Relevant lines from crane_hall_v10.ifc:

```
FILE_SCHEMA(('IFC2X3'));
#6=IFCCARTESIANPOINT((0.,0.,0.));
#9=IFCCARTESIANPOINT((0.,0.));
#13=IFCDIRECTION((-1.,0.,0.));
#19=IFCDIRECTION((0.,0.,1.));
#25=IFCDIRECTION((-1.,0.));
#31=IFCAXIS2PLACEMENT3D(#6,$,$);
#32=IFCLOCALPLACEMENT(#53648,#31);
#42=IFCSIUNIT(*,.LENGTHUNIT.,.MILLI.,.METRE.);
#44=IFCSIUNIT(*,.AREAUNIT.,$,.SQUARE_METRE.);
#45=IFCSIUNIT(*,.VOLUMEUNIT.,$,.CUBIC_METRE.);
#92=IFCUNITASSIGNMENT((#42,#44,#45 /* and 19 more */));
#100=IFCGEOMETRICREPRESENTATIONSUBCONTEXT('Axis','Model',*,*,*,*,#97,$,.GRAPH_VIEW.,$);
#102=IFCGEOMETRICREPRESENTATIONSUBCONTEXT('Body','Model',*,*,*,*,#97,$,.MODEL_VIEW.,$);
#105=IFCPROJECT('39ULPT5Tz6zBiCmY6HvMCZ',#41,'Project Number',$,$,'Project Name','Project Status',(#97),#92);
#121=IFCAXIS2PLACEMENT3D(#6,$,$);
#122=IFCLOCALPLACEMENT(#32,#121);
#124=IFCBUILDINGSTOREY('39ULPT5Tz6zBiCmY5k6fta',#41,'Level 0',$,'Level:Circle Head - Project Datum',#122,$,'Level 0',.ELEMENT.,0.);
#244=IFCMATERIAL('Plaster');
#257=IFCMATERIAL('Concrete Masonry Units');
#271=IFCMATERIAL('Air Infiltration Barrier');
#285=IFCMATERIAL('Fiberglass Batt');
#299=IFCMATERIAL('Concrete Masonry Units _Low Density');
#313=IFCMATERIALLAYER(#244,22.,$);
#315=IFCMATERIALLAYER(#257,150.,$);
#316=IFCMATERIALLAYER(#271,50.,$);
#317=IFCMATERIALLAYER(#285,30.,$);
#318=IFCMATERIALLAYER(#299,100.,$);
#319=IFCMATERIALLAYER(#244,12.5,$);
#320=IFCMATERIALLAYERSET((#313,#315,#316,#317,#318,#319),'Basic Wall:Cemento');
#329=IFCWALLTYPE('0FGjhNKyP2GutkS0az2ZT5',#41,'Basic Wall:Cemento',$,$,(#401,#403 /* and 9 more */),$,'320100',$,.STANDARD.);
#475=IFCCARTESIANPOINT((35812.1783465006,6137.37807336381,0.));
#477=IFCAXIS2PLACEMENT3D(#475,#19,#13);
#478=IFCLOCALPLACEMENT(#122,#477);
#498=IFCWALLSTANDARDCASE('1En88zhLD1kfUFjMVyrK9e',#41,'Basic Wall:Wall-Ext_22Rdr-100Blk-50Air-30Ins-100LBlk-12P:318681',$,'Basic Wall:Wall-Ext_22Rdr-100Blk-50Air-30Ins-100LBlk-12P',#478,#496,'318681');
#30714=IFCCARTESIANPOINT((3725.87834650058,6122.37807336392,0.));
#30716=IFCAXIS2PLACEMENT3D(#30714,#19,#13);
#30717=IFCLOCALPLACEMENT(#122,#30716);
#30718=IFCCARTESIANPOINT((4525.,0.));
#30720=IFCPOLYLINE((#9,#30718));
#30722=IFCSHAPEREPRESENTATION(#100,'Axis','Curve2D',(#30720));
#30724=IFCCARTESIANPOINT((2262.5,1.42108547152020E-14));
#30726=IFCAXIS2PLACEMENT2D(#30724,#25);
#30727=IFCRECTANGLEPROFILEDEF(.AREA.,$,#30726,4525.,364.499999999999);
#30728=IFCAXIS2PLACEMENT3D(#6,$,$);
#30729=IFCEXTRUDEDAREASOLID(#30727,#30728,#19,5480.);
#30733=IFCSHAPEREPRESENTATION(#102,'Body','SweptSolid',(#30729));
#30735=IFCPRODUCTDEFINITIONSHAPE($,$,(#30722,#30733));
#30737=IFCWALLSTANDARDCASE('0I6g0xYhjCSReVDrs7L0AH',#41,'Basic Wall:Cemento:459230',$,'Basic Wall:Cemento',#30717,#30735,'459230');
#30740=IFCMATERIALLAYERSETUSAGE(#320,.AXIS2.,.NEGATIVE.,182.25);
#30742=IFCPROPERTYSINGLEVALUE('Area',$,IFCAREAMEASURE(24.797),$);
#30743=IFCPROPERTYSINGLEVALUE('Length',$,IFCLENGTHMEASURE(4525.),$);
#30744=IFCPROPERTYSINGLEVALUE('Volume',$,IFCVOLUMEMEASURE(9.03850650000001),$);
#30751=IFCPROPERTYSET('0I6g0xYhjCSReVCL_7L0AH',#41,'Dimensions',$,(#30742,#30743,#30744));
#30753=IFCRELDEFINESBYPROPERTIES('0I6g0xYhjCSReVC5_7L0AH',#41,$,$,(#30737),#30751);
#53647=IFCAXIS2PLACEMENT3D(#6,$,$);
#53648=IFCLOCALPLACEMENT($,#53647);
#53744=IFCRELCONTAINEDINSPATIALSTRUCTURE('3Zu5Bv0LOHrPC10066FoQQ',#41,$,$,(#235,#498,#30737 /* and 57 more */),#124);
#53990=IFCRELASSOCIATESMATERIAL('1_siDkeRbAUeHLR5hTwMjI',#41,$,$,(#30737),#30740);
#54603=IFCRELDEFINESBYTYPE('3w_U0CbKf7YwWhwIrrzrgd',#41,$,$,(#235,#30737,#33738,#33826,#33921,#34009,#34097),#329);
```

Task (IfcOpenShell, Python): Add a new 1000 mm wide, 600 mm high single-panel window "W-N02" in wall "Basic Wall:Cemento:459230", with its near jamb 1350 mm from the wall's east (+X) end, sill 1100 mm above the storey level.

```python
import numpy as np
import ifcopenshell
import ifcopenshell.api.feature
import ifcopenshell.api.geometry
import ifcopenshell.api.pset
import ifcopenshell.api.root
import ifcopenshell.api.spatial
import ifcopenshell.api.type
import ifcopenshell.geom
import ifcopenshell.util.element
import ifcopenshell.util.placement
import ifcopenshell.util.representation
import ifcopenshell.util.shape
import ifcopenshell.util.unit

model = ifcopenshell.open("crane_hall_v10.ifc")
unit_scale = ifcopenshell.util.unit.calculate_unit_scale(model)
area_scale = ifcopenshell.util.unit.calculate_unit_scale(model, "AREAUNIT")
volume_scale = ifcopenshell.util.unit.calculate_unit_scale(model, "VOLUMEUNIT")
settings = ifcopenshell.geom.settings()


def volume(element):
    """Net volume in cubic metres, openings subtracted."""
    shape = ifcopenshell.geom.create_shape(settings, element)
    return ifcopenshell.util.shape.get_volume(shape.geometry)


wall = model.by_id(30737)
storey = ifcopenshell.util.element.get_container(wall, ifc_class="IfcBuildingStorey")
context = ifcopenshell.util.representation.get_context(model, "Model", "Body", "MODEL_VIEW")
before = volume(wall)

width, height, from_end, sill = 1, 0.6, 1.35, 1.1  # metres

# The wall runs along its own X axis, and the end named is its -X end.
wall_shape = ifcopenshell.geom.create_shape(settings, wall)
x, y, z = ifcopenshell.util.shape.get_vertices(wall_shape.geometry).T
start = x.min() + from_end
face, thickness = float(y.min()), float(y.max() - y.min())
wall_matrix = ifcopenshell.util.placement.get_local_placement(wall.ObjectPlacement)
level = ifcopenshell.util.placement.get_local_placement(storey.ObjectPlacement)[2, 3]


def in_wall(x, y):
    """Placement at x, y metres in the wall's axes, at sill height."""
    matrix = wall_matrix.copy()
    matrix[:, 3] = wall_matrix @ np.array([x / unit_scale, y / unit_scale, 0.0, 1.0])
    matrix[2, 3] = level + sill / unit_scale
    return matrix


# Opening: a box that overshoots both wall faces by 50 mm.
opening = ifcopenshell.api.root.create_entity(model, ifc_class="IfcOpeningElement")
box = ifcopenshell.api.geometry.add_wall_representation(
    model, context=context, length=width, height=height, thickness=thickness + 0.1
)
ifcopenshell.api.geometry.assign_representation(model, product=opening, representation=box)
ifcopenshell.api.geometry.edit_object_placement(model, product=opening, matrix=in_wall(start, face - 0.05), is_si=False)
ifcopenshell.api.feature.add_feature(model, feature=opening, element=wall)

window = ifcopenshell.api.root.create_entity(model, ifc_class="IfcWindow", name="W-N02")
window.OverallWidth, window.OverallHeight = width / unit_scale, height / unit_scale
body = ifcopenshell.api.geometry.add_window_representation(
    model,
    context=context,
    overall_width=window.OverallWidth,
    overall_height=window.OverallHeight,
    partition_type="SINGLE_PANEL",
)
ifcopenshell.api.geometry.assign_representation(model, product=window, representation=body)
ifcopenshell.api.spatial.assign_container(model, products=[window], relating_structure=storey)
fills = ifcopenshell.api.feature.add_filling(model, opening=opening, element=window)
fills.OwnerHistory = window.OwnerHistory  # required in IFC2X3

# IFC2X3 keeps the operation on the window style.
style = ifcopenshell.api.root.create_entity(model, ifc_class="IfcWindowStyle", name="W-N02")
style.OperationType, style.ConstructionType = "SINGLE_PANEL", "NOTDEFINED"
style.ParameterTakesPrecedence = style.Sizeable = False
ifcopenshell.api.type.assign_type(model, related_objects=[window], relating_type=style)

# Centre the window in the wall's thickness.
ifcopenshell.api.geometry.edit_object_placement(model, product=window, matrix=in_wall(start, face), is_si=False)
window_shape = ifcopenshell.geom.create_shape(settings, window)
depth = ifcopenshell.util.shape.get_vertices(window_shape.geometry)[:, 1]
offset = face + thickness / 2 - (depth.min() + depth.max()) / 2
ifcopenshell.api.geometry.edit_object_placement(model, product=window, matrix=in_wall(start, offset), is_si=False)

after = volume(wall)

# Update the wall's stored quantities.
pset = model.by_id(ifcopenshell.util.element.get_pset(wall, "Dimensions", should_inherit=False)["id"])
ifcopenshell.api.pset.edit_pset(model, pset=pset, properties={
    "Area": model.create_entity("IfcAreaMeasure", after / thickness / area_scale),
    "Volume": model.create_entity("IfcVolumeMeasure", after / volume_scale),
})

print(f"wall volume {before:.3f} -> {after:.3f} m3")

model.write("crane_hall_v10_edited.ifc")
```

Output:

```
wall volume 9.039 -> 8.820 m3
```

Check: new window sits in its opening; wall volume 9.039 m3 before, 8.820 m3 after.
